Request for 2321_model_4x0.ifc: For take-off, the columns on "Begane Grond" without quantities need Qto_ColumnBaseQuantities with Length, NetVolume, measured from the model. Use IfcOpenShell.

First a look at what the model holds.

```python
import ifcopenshell
import ifcopenshell.util.element
import ifcopenshell.util.unit

model = ifcopenshell.open("2321_model_4x0.ifc")
print(model.schema)
for unit_type in ("LENGTHUNIT", "AREAUNIT", "VOLUMEUNIT"):
    print(unit_type, ifcopenshell.util.unit.calculate_unit_scale(model, unit_type))
storey = next(s for s in model.by_type("IfcBuildingStorey") if s.Name == "Begane Grond")
columns = [e for e in ifcopenshell.util.element.get_decomposition(storey) if e.is_a("IfcColumn")]
for e in sorted(columns, key=lambda e: e.id()):
    print(e.id(), e.is_a(), e.Name, list(ifcopenshell.util.element.get_psets(e, qtos_only=True)), sep=" | ")
```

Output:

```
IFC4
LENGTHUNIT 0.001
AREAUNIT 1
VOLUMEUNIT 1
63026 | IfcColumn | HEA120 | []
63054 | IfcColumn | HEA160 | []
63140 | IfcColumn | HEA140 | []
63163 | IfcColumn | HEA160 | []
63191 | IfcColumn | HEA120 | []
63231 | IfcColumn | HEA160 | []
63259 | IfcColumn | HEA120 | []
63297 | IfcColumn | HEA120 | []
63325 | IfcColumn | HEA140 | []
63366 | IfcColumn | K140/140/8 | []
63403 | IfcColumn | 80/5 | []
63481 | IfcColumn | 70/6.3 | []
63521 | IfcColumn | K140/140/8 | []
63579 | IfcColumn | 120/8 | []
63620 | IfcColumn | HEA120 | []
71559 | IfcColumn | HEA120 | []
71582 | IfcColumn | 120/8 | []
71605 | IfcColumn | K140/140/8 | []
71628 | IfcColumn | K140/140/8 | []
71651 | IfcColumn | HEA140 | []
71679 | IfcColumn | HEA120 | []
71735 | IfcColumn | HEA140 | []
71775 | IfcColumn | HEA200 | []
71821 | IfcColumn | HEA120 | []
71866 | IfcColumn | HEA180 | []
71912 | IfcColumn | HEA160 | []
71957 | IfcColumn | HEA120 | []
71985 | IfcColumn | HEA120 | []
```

```python
import ifcopenshell
import ifcopenshell.api.pset
import ifcopenshell.geom
import ifcopenshell.util.element
import ifcopenshell.util.shape
import ifcopenshell.util.unit

model = ifcopenshell.open("2321_model_4x0.ifc")
unit_scale = ifcopenshell.util.unit.calculate_unit_scale(model)
volume_scale = ifcopenshell.util.unit.calculate_unit_scale(model, "VOLUMEUNIT")
settings = ifcopenshell.geom.settings()

storey = next(s for s in model.by_type("IfcBuildingStorey") if s.Name == "Begane Grond")
columns = [e for e in ifcopenshell.util.element.get_decomposition(storey) if e.is_a("IfcColumn")]

for e in sorted(columns, key=lambda e: e.id()):
    if ifcopenshell.util.element.get_psets(e, qtos_only=True, should_inherit=False):
        continue
    # Geometry comes back in metres, in the element's own axes.
    shape = ifcopenshell.geom.create_shape(settings, e)
    values = {
        "Length": ifcopenshell.util.shape.get_z(shape.geometry) / unit_scale,
        "NetVolume": ifcopenshell.util.shape.get_volume(shape.geometry) / volume_scale,
    }
    qto = ifcopenshell.api.pset.add_qto(model, product=e, name="Qto_ColumnBaseQuantities")
    ifcopenshell.api.pset.edit_qto(model, qto=qto, properties=values)
    print(e.id(), {k: round(v, 3) for k, v in values.items()})

model.write("2321_model_4x0_edited.ifc")
```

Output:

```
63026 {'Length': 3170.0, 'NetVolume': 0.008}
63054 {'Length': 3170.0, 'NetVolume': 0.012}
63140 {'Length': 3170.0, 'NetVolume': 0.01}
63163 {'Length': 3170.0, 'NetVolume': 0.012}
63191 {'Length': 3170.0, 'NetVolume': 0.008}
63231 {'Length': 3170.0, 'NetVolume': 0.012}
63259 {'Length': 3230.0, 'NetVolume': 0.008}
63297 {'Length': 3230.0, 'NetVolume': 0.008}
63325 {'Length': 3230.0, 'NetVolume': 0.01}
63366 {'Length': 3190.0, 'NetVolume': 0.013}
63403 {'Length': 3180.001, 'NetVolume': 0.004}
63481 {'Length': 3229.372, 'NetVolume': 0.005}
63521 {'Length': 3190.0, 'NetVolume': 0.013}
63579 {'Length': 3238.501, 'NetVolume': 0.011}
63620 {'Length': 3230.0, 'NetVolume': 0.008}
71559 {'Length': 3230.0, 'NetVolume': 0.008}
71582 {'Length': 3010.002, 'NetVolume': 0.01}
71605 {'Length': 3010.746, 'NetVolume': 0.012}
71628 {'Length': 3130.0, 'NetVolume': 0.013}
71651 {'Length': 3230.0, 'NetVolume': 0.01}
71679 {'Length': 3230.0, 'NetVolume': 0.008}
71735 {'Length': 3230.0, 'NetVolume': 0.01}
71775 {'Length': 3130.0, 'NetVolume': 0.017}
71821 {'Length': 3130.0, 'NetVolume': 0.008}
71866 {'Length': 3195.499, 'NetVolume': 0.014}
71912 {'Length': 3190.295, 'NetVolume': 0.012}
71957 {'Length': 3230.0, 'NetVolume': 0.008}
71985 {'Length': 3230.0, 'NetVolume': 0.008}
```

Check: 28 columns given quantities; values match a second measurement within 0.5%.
